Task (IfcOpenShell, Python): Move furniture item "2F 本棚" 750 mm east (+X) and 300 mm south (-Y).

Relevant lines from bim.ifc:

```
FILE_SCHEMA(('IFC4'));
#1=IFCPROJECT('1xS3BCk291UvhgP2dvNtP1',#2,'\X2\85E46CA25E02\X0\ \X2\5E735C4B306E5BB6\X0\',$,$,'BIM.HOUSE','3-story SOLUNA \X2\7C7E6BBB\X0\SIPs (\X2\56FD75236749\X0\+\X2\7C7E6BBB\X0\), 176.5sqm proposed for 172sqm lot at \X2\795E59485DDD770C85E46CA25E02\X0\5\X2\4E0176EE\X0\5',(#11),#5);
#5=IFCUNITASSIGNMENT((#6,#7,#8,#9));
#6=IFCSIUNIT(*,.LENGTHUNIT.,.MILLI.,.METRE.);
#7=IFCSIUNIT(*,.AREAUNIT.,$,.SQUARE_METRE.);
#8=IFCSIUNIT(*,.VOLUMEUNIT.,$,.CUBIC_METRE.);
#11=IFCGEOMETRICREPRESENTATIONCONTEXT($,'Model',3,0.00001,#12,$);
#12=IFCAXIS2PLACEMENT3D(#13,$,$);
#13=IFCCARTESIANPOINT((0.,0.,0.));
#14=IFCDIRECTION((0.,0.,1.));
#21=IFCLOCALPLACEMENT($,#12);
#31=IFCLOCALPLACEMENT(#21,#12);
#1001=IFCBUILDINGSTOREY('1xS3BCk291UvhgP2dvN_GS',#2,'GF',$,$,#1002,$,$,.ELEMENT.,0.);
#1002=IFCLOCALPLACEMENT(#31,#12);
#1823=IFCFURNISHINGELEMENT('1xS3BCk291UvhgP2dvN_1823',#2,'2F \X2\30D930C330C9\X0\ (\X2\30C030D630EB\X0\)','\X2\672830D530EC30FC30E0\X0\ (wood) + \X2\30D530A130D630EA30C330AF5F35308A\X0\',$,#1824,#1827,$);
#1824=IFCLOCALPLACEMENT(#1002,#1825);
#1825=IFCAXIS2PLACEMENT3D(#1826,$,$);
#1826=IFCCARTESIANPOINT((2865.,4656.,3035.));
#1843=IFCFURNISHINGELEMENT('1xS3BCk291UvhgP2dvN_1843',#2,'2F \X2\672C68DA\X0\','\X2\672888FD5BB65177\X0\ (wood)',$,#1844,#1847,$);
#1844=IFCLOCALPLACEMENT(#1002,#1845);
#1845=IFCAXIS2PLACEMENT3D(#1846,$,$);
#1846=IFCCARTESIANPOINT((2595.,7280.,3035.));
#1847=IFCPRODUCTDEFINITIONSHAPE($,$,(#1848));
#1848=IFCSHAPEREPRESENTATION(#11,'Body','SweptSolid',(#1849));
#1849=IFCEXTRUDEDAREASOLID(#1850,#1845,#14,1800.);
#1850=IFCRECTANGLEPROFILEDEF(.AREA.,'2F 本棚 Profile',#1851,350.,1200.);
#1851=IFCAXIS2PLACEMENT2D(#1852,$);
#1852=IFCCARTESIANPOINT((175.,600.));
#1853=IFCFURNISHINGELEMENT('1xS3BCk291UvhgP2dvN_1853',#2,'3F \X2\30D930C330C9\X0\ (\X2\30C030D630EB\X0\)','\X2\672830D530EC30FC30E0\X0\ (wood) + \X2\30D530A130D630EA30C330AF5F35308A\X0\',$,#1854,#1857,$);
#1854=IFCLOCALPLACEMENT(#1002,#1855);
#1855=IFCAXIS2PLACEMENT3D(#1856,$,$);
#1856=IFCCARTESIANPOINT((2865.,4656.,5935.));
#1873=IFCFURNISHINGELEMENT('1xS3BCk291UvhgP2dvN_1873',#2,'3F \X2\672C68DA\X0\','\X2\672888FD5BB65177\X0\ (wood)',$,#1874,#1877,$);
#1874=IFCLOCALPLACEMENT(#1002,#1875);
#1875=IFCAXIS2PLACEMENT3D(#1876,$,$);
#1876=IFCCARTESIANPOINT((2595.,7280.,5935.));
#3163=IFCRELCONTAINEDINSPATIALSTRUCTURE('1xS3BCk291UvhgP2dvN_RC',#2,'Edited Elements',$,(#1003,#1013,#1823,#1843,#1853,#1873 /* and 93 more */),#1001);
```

```python
import ifcopenshell
import ifcopenshell.api.geometry
import ifcopenshell.util.placement

model = ifcopenshell.open("bim.ifc")

item = model.by_guid("1xS3BCk291UvhgP2dvN_1843")
matrix = ifcopenshell.util.placement.get_local_placement(item.ObjectPlacement)
matrix[0, 3] += 750.0
matrix[1, 3] -= 300.0
ifcopenshell.api.geometry.edit_object_placement(model, product=item, matrix=matrix, is_si=False)

print(ifcopenshell.util.placement.get_local_placement(item.ObjectPlacement).round(3) + 0.0)

model.write("bim_rev.ifc")
```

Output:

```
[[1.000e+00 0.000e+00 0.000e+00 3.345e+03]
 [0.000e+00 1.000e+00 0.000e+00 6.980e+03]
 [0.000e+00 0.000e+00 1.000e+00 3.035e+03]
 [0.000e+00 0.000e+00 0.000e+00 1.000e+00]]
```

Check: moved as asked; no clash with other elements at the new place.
